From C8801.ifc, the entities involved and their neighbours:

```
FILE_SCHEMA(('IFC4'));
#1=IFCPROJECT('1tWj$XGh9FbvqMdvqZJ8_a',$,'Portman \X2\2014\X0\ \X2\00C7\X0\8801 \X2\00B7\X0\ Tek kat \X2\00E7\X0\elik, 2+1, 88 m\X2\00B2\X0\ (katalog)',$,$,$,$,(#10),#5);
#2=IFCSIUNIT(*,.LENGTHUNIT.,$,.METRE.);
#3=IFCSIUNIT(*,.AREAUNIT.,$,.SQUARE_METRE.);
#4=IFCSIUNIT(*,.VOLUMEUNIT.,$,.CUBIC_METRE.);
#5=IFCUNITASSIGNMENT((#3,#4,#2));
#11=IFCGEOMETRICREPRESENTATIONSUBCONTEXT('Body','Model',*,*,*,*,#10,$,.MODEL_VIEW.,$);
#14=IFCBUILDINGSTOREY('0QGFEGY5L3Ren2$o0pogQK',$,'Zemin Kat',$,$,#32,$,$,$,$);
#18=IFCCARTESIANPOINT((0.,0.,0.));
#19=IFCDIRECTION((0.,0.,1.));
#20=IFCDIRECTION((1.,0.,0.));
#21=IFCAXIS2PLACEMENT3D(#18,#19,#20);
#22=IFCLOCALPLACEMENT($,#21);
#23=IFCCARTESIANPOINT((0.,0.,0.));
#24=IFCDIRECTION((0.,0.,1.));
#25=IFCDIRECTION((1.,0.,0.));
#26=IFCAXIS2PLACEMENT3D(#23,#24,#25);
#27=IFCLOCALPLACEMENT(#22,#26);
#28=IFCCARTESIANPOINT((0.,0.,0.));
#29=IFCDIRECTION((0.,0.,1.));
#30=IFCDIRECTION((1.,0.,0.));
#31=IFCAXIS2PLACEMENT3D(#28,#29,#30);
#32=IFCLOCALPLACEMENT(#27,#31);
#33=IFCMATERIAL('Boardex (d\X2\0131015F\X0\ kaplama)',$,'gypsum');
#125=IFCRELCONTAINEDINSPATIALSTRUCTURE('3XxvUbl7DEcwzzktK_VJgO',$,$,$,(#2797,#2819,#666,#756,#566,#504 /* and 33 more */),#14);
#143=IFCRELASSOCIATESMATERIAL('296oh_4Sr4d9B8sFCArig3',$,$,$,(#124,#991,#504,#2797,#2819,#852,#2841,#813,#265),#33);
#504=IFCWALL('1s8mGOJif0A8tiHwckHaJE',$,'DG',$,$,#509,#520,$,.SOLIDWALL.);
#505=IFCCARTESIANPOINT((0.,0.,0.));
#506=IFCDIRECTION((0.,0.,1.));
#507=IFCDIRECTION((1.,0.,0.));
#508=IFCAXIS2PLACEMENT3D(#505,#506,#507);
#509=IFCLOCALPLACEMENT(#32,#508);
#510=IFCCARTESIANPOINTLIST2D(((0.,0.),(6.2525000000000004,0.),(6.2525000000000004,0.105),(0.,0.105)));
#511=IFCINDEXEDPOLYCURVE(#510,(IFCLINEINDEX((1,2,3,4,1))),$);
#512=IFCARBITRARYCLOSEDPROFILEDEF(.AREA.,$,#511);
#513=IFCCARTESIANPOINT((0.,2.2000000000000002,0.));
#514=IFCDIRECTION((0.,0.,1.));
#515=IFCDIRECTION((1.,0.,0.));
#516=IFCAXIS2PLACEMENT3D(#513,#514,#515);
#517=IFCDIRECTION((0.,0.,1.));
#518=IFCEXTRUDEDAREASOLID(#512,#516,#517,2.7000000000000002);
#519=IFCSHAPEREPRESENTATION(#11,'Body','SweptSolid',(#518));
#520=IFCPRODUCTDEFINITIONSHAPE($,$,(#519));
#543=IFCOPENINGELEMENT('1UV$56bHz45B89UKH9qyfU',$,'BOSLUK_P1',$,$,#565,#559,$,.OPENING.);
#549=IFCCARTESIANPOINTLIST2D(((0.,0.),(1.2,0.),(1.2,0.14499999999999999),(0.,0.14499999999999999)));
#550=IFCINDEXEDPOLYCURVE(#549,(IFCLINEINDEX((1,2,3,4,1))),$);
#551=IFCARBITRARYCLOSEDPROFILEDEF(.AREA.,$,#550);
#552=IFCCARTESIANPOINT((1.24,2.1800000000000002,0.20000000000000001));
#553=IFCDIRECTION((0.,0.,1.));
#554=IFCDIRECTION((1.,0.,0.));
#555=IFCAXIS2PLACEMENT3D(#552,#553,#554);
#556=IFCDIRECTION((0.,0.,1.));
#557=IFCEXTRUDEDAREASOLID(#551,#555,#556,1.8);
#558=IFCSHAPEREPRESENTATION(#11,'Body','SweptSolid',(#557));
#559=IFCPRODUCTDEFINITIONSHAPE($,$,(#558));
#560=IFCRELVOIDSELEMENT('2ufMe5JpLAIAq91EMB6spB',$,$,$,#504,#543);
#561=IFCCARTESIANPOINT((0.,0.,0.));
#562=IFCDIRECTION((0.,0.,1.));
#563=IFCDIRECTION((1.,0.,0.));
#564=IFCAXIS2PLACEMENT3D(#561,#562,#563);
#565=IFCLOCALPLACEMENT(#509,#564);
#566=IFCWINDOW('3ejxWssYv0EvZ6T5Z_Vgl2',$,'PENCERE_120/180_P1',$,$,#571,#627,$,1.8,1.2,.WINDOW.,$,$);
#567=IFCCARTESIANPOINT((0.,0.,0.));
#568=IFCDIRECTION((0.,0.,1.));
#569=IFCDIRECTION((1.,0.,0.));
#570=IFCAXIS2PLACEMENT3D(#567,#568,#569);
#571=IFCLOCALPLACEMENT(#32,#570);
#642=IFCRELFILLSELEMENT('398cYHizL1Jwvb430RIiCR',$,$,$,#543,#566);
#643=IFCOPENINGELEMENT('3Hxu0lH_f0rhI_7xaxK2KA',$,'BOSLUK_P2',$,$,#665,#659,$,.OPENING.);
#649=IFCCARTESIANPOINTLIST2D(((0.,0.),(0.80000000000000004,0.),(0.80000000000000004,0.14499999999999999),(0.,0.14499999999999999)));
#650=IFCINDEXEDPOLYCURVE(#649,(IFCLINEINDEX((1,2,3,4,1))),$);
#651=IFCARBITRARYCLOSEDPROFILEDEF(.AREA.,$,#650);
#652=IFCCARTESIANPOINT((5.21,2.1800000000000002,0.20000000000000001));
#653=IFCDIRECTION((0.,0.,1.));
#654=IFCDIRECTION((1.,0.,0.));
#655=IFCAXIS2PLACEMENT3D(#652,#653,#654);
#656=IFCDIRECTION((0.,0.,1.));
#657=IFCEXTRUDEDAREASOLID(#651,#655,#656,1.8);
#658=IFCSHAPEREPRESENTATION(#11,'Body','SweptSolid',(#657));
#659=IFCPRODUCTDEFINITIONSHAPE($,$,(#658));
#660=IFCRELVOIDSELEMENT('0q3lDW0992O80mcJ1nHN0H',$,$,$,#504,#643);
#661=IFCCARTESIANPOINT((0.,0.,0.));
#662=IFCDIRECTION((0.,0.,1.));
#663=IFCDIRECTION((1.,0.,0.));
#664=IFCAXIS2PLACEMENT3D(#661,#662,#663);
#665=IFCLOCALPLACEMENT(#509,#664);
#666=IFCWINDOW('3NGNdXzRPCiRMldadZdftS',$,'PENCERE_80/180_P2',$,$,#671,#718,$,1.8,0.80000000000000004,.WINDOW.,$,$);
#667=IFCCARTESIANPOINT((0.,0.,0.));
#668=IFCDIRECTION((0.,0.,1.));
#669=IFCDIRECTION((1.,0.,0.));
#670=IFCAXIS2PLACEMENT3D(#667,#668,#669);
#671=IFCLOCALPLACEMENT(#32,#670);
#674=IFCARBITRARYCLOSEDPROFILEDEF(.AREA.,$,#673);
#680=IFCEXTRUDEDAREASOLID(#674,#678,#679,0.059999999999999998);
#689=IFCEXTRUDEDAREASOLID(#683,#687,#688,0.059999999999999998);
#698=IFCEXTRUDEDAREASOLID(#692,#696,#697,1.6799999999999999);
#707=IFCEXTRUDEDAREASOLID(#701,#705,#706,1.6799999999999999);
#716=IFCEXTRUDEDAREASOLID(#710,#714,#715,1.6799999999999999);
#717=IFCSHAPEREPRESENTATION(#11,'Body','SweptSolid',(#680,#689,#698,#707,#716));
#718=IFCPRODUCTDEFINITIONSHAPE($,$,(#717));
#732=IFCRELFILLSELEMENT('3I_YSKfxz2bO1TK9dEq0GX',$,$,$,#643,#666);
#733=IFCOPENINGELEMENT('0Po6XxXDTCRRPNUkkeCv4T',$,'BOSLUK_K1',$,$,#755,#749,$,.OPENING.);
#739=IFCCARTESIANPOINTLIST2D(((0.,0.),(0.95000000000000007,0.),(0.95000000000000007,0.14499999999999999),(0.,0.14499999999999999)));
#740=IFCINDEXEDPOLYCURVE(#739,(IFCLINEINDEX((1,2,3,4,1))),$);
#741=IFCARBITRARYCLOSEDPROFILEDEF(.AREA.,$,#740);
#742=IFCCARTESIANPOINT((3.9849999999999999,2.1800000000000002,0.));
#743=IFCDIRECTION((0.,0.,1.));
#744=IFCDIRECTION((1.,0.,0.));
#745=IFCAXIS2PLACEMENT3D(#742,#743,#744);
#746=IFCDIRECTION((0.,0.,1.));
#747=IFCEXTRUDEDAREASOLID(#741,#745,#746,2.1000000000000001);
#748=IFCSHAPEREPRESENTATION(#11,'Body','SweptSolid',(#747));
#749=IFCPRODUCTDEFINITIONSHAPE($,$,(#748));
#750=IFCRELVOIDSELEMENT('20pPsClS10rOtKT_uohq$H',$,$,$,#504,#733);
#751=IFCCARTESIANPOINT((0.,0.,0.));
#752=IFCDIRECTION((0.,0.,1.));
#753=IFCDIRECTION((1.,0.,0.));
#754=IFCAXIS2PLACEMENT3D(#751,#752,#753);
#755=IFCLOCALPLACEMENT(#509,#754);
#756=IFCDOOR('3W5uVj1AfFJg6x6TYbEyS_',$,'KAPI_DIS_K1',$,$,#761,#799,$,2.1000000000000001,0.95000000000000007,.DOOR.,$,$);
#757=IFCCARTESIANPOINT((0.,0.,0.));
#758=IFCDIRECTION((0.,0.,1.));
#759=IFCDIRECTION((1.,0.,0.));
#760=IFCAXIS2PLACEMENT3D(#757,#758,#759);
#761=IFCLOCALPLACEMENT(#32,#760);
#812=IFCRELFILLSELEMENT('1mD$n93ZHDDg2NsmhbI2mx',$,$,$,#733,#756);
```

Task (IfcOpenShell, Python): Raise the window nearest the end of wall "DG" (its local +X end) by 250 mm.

```python
import numpy as np
import ifcopenshell
import ifcopenshell.api.geometry
import ifcopenshell.util.placement
import ifcopenshell.util.unit

model = ifcopenshell.open("C8801.ifc")
unit_scale = ifcopenshell.util.unit.calculate_unit_scale(model)

window = model.by_guid("3NGNdXzRPCiRMldadZdftS")
opening = window.FillsVoids[0].RelatingOpeningElement
dz = 0.25 / unit_scale

shift = np.array([0.0, 0.0, dz])
# The window is not placed relative to its opening, so move both.
for product in (opening, window):
    matrix = ifcopenshell.util.placement.get_local_placement(product.ObjectPlacement)
    matrix[:3, 3] += shift
    ifcopenshell.api.geometry.edit_object_placement(model, product=product, matrix=matrix, is_si=False)

print(f"moved by {dz * unit_scale:+.3f} m")

model.write("C8801_rev.ifc")
```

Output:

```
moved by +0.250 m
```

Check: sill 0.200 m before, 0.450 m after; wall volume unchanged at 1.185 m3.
